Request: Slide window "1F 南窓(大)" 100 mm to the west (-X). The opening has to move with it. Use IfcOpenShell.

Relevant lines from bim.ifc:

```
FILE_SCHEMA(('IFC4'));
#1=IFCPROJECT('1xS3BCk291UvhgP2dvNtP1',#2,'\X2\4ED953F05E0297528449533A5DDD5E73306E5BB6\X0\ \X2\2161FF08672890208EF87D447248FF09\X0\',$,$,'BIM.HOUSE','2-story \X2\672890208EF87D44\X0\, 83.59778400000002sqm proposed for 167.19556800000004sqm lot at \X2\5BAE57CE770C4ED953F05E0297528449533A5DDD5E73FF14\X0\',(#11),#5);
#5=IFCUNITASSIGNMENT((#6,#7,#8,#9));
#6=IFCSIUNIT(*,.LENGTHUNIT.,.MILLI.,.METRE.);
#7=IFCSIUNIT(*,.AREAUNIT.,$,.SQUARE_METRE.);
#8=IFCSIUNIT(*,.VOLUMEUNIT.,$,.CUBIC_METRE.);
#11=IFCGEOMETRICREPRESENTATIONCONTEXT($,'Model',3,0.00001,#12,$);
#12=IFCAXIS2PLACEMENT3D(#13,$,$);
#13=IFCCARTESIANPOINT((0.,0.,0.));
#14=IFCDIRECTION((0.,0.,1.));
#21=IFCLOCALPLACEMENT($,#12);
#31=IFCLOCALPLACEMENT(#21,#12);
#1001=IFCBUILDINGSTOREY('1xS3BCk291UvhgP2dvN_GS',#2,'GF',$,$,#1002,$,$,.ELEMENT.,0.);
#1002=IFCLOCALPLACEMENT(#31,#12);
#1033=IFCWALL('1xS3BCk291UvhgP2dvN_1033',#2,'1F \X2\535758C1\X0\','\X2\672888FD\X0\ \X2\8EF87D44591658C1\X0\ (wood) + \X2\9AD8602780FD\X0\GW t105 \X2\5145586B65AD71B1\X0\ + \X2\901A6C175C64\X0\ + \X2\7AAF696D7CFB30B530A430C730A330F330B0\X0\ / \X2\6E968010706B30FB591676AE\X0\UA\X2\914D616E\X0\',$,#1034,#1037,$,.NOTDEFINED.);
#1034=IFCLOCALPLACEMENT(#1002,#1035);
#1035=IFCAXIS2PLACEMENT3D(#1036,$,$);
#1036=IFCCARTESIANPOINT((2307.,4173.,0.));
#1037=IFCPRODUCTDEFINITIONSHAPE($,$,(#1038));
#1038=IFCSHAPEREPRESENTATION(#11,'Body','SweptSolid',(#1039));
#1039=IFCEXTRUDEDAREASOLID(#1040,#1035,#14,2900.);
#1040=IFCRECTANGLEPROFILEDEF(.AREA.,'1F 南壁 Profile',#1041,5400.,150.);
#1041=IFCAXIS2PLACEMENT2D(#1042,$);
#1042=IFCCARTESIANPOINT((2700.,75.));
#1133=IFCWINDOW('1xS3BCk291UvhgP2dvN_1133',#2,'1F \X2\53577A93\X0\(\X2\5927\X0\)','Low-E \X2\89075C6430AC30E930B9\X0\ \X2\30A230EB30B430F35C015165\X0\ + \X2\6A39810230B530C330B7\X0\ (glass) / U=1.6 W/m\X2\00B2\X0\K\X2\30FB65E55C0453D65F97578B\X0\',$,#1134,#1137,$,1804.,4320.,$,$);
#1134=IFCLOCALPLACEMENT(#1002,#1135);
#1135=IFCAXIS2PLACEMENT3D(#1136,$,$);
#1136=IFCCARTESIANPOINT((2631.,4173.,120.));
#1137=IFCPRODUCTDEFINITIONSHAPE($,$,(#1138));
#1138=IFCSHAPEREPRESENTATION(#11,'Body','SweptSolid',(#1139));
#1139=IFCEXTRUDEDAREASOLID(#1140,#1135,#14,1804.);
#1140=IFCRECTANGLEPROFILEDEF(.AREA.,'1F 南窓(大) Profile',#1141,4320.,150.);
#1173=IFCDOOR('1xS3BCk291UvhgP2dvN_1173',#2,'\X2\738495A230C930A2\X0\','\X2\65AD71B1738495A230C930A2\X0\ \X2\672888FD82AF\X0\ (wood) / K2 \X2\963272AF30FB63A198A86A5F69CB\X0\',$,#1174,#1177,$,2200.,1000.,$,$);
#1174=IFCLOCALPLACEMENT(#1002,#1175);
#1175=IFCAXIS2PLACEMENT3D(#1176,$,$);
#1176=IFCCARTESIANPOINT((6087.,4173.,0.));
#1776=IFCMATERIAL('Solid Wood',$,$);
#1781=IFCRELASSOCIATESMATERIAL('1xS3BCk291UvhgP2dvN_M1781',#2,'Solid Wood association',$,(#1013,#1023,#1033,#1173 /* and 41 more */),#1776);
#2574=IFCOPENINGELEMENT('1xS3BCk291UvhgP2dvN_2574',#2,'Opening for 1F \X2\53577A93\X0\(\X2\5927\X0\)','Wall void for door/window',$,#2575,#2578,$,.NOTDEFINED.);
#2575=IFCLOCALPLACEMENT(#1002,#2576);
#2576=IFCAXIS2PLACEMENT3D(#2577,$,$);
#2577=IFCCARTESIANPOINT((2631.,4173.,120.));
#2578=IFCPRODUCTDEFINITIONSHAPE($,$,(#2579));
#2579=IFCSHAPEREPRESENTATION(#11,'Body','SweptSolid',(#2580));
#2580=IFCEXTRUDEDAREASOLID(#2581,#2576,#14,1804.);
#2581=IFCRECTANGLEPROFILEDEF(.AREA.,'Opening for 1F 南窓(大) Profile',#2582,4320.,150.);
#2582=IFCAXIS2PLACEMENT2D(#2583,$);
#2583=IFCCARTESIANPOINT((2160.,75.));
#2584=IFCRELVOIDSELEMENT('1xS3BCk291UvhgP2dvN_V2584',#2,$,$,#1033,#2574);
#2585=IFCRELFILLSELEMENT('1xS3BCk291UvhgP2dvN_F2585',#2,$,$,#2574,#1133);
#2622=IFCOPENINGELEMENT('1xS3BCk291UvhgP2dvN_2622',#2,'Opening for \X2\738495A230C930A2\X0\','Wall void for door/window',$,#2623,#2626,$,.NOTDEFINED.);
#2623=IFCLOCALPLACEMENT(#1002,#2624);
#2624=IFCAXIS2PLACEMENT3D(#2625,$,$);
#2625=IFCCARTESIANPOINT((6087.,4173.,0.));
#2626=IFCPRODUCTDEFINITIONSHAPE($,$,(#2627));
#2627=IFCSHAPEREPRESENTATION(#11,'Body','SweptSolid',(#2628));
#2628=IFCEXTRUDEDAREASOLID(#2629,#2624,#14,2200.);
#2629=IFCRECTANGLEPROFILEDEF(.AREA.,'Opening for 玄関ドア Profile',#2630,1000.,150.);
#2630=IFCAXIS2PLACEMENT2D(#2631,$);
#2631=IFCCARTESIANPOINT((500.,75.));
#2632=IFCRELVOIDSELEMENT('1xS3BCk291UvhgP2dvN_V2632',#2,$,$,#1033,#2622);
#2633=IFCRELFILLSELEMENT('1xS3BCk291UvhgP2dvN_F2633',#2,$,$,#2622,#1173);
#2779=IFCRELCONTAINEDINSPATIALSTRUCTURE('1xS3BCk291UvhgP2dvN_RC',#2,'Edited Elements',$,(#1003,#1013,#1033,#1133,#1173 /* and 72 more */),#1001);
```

```python
import ifcopenshell
import ifcopenshell.api.geometry
import ifcopenshell.util.placement
import ifcopenshell.util.unit

model = ifcopenshell.open("bim.ifc")
unit_scale = ifcopenshell.util.unit.calculate_unit_scale(model)

window = model.by_id(1133)
opening = window.FillsVoids[0].RelatingOpeningElement
wall = opening.VoidsElements[0].RelatingBuildingElement

wall_matrix = ifcopenshell.util.placement.get_local_placement(wall.ObjectPlacement)
shift = wall_matrix[:3, 0] * -0.1 / unit_scale
before = ifcopenshell.util.placement.get_local_placement(window.ObjectPlacement)[:3, 3].copy()

# The window is not placed relative to its opening, so move both.
for product in (opening, window):
    matrix = ifcopenshell.util.placement.get_local_placement(product.ObjectPlacement)
    matrix[:3, 3] += shift
    ifcopenshell.api.geometry.edit_object_placement(model, product=product, matrix=matrix, is_si=False)

after = ifcopenshell.util.placement.get_local_placement(window.ObjectPlacement)[:3, 3]
print("window moved by", (after - before).round(3) + 0.0)

model.write("bim-out.ifc")
```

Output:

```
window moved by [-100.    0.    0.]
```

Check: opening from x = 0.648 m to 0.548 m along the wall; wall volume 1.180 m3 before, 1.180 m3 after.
